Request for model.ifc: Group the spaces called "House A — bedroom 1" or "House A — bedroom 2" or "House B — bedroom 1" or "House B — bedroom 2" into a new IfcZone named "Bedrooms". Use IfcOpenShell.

First a look at what the model holds.

```python
import ifcopenshell

model = ifcopenshell.open("model.ifc")
print(model.schema)
seen = {}
for space in model.by_type("IfcSpace"):
    seen[space.Name] = seen.get(space.Name, 0) + 1
for name, count in sorted(seen.items(), key=str):
    print(count, "x", name)
print("zones:", [z.Name for z in model.by_type("IfcZone")][:20])
```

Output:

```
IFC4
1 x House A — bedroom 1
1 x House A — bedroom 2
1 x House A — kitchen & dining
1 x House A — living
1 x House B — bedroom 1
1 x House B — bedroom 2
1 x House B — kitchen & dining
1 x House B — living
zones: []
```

```python
import ifcopenshell
import ifcopenshell.api.group
import ifcopenshell.api.root

model = ifcopenshell.open("model.ifc")

names = {"House A — bedroom 1", "House A — bedroom 2", "House B — bedroom 1", "House B — bedroom 2"}
spaces = [s for s in model.by_type("IfcSpace") if s.Name in names]

zone = ifcopenshell.api.root.create_entity(model, ifc_class="IfcZone", name="Bedrooms")
ifcopenshell.api.group.assign_group(model, products=spaces, group=zone)
print(len(spaces), "spaces in", zone.Name)

model.write("model_v2.ifc")
```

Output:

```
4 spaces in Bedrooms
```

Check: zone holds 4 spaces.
